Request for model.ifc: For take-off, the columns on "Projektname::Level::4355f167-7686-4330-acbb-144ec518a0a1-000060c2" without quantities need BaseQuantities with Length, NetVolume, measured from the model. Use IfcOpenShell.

First a look at what the model holds.

```python
import ifcopenshell
import ifcopenshell.util.element
import ifcopenshell.util.unit

model = ifcopenshell.open("model.ifc")
print(model.schema)
for unit_type in ("LENGTHUNIT", "AREAUNIT", "VOLUMEUNIT"):
    print(unit_type, ifcopenshell.util.unit.calculate_unit_scale(model, unit_type))
storey = next(s for s in model.by_type("IfcBuildingStorey") if s.Name == "Projektname::Level::4355f167-7686-4330-acbb-144ec518a0a1-000060c2")
columns = [e for e in ifcopenshell.util.element.get_decomposition(storey) if e.is_a("IfcColumn")]
for e in sorted(columns, key=lambda e: e.id()):
    print(e.id(), e.is_a(), e.Name, list(ifcopenshell.util.element.get_psets(e, qtos_only=True)), sep=" | ")
```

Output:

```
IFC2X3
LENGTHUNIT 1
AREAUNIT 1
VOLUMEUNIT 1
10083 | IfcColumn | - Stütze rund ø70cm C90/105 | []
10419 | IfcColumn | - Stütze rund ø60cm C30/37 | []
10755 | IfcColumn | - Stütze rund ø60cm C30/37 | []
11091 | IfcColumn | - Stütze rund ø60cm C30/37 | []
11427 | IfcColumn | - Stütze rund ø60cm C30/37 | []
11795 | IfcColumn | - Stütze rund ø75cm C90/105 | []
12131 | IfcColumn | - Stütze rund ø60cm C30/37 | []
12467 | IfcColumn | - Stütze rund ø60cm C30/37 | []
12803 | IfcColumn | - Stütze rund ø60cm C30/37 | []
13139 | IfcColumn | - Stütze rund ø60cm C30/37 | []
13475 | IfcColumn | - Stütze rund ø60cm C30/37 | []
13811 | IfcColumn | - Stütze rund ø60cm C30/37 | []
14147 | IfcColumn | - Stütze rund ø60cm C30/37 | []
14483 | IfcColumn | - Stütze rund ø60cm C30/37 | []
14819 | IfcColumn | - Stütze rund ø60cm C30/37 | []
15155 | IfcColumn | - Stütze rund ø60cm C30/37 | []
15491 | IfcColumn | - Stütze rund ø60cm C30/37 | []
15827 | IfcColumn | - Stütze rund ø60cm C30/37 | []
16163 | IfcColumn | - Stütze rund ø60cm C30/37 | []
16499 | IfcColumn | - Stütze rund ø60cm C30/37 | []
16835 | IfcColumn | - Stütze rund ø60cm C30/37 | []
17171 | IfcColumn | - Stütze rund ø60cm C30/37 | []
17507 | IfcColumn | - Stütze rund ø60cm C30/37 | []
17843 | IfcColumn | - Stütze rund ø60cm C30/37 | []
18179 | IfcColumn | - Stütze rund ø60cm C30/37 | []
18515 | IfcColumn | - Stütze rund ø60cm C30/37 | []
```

```python
import ifcopenshell
import ifcopenshell.api.pset
import ifcopenshell.geom
import ifcopenshell.util.element
import ifcopenshell.util.shape
import ifcopenshell.util.unit

model = ifcopenshell.open("model.ifc")
unit_scale = ifcopenshell.util.unit.calculate_unit_scale(model)
volume_scale = ifcopenshell.util.unit.calculate_unit_scale(model, "VOLUMEUNIT")
settings = ifcopenshell.geom.settings()

storey = next(s for s in model.by_type("IfcBuildingStorey") if s.Name == "Projektname::Level::4355f167-7686-4330-acbb-144ec518a0a1-000060c2")
columns = [e for e in ifcopenshell.util.element.get_decomposition(storey) if e.is_a("IfcColumn")]

for e in sorted(columns, key=lambda e: e.id()):
    if ifcopenshell.util.element.get_psets(e, qtos_only=True, should_inherit=False):
        continue
    # Geometry comes back in metres, in the element's own axes.
    shape = ifcopenshell.geom.create_shape(settings, e)
    values = {
        "Length": ifcopenshell.util.shape.get_z(shape.geometry) / unit_scale,
        "NetVolume": ifcopenshell.util.shape.get_volume(shape.geometry) / volume_scale,
    }
    qto = ifcopenshell.api.pset.add_qto(model, product=e, name="BaseQuantities")
    ifcopenshell.api.pset.edit_qto(model, qto=qto, properties=values)
    print(e.id(), {k: round(v, 3) for k, v in values.items()})

model.write("model_edited.ifc")
```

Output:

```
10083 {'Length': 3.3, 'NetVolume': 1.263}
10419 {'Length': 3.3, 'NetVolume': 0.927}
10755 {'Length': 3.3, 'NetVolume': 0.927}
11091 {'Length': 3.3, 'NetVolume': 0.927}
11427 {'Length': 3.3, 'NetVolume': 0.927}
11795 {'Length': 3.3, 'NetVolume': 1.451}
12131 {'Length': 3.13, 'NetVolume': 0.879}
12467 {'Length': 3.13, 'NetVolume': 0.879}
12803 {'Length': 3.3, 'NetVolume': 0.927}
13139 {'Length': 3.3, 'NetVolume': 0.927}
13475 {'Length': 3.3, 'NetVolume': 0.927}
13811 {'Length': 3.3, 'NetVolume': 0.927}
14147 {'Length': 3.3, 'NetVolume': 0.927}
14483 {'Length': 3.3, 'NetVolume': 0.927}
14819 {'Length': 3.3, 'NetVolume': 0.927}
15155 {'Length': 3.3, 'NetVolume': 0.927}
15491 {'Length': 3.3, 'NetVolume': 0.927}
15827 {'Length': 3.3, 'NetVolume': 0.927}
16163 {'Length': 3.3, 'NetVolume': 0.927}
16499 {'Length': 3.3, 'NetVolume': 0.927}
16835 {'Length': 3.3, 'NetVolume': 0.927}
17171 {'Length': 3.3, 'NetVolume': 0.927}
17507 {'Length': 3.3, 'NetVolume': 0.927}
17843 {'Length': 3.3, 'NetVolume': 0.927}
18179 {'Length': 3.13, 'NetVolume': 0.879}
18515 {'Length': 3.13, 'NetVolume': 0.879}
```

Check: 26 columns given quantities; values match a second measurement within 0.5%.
